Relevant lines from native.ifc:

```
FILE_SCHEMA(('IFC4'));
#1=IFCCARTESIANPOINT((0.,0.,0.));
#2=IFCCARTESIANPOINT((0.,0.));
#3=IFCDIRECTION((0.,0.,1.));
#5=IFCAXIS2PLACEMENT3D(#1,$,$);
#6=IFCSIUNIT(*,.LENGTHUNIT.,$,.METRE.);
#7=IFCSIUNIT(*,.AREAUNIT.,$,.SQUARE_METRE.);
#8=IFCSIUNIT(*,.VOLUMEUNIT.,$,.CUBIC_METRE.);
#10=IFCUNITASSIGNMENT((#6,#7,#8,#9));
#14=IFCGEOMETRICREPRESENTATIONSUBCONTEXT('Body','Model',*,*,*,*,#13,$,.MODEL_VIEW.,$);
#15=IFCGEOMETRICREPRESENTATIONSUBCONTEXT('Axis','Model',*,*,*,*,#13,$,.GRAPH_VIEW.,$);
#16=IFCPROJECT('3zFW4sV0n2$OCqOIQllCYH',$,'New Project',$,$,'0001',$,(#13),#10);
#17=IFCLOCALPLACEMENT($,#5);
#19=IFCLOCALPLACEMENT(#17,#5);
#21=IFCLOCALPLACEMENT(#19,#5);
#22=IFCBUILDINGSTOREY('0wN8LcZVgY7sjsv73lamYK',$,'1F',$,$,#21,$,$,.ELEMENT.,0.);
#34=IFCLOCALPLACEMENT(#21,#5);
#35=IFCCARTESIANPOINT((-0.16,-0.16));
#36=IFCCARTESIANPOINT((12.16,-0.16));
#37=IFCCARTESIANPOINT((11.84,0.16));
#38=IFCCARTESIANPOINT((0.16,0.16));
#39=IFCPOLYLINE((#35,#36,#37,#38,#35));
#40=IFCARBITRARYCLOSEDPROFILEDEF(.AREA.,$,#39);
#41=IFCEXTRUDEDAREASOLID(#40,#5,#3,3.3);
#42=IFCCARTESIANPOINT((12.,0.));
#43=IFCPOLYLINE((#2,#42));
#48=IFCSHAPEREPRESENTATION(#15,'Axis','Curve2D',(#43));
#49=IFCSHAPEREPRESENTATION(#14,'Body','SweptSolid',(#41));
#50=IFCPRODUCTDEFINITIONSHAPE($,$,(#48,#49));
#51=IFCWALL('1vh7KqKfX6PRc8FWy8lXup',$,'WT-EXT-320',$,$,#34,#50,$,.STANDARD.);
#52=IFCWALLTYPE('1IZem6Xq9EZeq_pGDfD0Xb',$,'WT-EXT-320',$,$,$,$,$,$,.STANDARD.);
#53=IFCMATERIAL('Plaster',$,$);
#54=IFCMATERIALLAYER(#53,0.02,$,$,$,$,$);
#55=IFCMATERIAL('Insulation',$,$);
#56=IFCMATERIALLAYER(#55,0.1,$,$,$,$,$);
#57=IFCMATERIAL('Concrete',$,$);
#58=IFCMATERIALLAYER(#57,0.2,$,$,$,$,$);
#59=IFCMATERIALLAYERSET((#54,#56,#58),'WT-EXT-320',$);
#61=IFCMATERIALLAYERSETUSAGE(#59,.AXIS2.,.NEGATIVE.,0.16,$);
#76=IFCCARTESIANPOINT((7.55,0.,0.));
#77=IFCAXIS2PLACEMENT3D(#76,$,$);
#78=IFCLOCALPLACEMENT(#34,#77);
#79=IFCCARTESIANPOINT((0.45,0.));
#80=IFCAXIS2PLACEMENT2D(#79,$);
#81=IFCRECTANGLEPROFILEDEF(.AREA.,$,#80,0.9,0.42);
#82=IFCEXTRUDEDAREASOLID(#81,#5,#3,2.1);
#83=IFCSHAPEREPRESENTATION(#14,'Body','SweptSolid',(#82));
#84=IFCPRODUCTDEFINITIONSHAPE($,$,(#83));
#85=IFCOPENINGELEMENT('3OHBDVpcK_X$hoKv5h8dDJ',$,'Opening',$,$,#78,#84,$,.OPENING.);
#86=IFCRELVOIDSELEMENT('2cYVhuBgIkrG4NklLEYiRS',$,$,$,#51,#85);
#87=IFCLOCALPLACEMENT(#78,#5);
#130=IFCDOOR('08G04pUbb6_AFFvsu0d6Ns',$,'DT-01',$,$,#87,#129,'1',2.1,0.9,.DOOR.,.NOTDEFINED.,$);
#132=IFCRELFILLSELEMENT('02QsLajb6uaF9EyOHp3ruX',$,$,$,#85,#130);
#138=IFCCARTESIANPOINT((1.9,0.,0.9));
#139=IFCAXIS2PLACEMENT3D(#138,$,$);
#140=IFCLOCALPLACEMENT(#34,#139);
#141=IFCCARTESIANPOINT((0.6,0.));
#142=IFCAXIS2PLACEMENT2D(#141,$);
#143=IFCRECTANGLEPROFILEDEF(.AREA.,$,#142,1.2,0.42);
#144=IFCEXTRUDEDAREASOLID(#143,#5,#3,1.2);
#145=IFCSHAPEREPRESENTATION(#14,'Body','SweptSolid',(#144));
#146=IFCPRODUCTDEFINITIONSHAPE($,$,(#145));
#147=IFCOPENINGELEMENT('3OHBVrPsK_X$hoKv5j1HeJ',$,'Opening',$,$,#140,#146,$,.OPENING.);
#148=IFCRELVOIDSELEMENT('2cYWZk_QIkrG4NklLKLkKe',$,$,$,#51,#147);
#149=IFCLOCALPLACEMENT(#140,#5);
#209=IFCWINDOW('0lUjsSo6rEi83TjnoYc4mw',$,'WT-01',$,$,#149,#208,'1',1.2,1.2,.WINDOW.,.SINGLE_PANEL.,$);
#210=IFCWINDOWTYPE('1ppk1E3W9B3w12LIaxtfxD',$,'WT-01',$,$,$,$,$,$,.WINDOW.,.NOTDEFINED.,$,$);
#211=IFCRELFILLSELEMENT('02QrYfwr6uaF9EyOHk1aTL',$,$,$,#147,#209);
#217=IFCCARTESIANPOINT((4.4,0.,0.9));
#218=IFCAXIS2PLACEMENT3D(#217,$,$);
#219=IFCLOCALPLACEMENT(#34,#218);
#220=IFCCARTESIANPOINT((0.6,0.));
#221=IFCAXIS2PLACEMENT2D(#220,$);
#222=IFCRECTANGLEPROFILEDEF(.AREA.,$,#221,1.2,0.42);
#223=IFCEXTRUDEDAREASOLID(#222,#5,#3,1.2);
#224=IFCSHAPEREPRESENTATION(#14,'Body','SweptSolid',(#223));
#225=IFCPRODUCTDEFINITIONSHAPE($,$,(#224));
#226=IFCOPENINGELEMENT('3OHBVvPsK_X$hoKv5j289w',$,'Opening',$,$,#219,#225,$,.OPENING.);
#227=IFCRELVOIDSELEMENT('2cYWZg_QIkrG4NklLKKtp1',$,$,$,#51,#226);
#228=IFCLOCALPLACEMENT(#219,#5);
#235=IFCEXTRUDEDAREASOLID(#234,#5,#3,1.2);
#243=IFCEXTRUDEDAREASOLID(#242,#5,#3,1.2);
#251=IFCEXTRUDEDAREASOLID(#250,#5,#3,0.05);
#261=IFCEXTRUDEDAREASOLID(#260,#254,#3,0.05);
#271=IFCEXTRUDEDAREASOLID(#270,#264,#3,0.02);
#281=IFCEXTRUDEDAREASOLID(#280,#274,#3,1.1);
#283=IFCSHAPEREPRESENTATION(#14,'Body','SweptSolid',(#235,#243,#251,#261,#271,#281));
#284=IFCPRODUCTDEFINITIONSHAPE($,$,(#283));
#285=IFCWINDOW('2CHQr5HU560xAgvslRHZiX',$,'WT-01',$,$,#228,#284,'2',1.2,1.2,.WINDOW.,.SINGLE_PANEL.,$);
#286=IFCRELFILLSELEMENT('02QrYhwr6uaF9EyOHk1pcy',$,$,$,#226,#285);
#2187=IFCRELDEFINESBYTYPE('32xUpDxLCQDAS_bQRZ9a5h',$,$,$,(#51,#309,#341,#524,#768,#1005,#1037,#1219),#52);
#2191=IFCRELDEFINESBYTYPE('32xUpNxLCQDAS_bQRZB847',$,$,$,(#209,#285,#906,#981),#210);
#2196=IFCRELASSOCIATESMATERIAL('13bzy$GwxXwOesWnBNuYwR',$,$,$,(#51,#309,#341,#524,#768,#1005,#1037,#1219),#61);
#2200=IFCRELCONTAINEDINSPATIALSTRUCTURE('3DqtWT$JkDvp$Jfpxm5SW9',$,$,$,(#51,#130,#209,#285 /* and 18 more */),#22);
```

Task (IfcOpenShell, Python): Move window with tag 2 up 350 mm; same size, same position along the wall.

```python
import numpy as np
import ifcopenshell
import ifcopenshell.api.geometry
import ifcopenshell.util.placement
import ifcopenshell.util.unit

model = ifcopenshell.open("native.ifc")
unit_scale = ifcopenshell.util.unit.calculate_unit_scale(model)

window = model.by_guid("2CHQr5HU560xAgvslRHZiX")
opening = window.FillsVoids[0].RelatingOpeningElement
dz = 0.35 / unit_scale

shift = np.array([0.0, 0.0, dz])
# The window is placed relative to its opening, so it follows when the opening moves.
matrix = ifcopenshell.util.placement.get_local_placement(opening.ObjectPlacement)
matrix[:3, 3] += shift
ifcopenshell.api.geometry.edit_object_placement(
    model, product=opening, matrix=matrix, is_si=False, should_transform_children=True
)

print(f"moved by {dz * unit_scale:+.3f} m")

model.write("native-out.ifc")
```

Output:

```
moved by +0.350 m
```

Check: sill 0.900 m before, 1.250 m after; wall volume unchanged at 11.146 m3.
